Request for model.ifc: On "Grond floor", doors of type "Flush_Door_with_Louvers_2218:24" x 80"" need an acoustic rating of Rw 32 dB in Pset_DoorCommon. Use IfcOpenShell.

First a look at what the model holds.

```python
import ifcopenshell
import ifcopenshell.util.element

model = ifcopenshell.open("model.ifc")
print(model.schema)
storey = next(s for s in model.by_type("IfcBuildingStorey") if s.Name == "Grond floor")
doors = [e for e in ifcopenshell.util.element.get_decomposition(storey) if e.is_a("IfcDoor")]
seen = {}
for e in doors:
    element_type = ifcopenshell.util.element.get_type(e)
    key = (element_type.Name if element_type != e and element_type else None, ifcopenshell.util.element.get_pset(e, "Pset_DoorCommon", "AcousticRating"))
    seen[key] = seen.get(key, 0) + 1
for (name, value), count in sorted(seen.items(), key=str):
    print(count, "x", name, "|", value)
```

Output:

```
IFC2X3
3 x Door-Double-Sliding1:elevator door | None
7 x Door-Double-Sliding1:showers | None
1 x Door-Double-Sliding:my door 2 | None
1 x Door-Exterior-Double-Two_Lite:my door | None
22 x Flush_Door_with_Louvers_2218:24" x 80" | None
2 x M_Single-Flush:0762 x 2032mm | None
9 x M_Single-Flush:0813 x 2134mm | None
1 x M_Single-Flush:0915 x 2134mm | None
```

```python
import ifcopenshell
import ifcopenshell.api.pset
import ifcopenshell.util.element

model = ifcopenshell.open("model.ifc")

storey = next(s for s in model.by_type("IfcBuildingStorey") if s.Name == "Grond floor")
doors = [e for e in ifcopenshell.util.element.get_decomposition(storey) if e.is_a("IfcDoor")]

count = 0
for e in doors:
    element_type = ifcopenshell.util.element.get_type(e)
    if element_type in (None, e) or element_type.Name != 'Flush_Door_with_Louvers_2218:24" x 80"':
        continue
    # add_pset returns the element's existing set when there is one.
    pset = ifcopenshell.api.pset.add_pset(model, product=e, name="Pset_DoorCommon")
    ifcopenshell.api.pset.edit_pset(model, pset=pset, properties={"AcousticRating": "Rw 32 dB"})
    count += 1

print(count, "doors updated")

model.write("model_updated.ifc")
```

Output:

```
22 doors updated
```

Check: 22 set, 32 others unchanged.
